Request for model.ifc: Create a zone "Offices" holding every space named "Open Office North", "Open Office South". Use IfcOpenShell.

First a look at what the model holds.

```python
import ifcopenshell

model = ifcopenshell.open("model.ifc")
print(model.schema)
seen = {}
for space in model.by_type("IfcSpace"):
    seen[space.LongName] = seen.get(space.LongName, 0) + 1
for name, count in sorted(seen.items(), key=str):
    print(count, "x", name)
print("zones:", [z.Name for z in model.by_type("IfcZone")][:20])
```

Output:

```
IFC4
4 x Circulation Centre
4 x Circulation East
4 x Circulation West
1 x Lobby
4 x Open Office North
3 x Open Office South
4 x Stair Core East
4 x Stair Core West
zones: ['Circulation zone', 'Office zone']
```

```python
import ifcopenshell
import ifcopenshell.api.group
import ifcopenshell.api.root

model = ifcopenshell.open("model.ifc")

names = {"Open Office North", "Open Office South"}
spaces = [s for s in model.by_type("IfcSpace") if s.LongName in names]

zone = ifcopenshell.api.root.create_entity(model, ifc_class="IfcZone", name="Offices")
ifcopenshell.api.group.assign_group(model, products=spaces, group=zone)
print(len(spaces), "spaces in", zone.Name)

model.write("model_updated.ifc")
```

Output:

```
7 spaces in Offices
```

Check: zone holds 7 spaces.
